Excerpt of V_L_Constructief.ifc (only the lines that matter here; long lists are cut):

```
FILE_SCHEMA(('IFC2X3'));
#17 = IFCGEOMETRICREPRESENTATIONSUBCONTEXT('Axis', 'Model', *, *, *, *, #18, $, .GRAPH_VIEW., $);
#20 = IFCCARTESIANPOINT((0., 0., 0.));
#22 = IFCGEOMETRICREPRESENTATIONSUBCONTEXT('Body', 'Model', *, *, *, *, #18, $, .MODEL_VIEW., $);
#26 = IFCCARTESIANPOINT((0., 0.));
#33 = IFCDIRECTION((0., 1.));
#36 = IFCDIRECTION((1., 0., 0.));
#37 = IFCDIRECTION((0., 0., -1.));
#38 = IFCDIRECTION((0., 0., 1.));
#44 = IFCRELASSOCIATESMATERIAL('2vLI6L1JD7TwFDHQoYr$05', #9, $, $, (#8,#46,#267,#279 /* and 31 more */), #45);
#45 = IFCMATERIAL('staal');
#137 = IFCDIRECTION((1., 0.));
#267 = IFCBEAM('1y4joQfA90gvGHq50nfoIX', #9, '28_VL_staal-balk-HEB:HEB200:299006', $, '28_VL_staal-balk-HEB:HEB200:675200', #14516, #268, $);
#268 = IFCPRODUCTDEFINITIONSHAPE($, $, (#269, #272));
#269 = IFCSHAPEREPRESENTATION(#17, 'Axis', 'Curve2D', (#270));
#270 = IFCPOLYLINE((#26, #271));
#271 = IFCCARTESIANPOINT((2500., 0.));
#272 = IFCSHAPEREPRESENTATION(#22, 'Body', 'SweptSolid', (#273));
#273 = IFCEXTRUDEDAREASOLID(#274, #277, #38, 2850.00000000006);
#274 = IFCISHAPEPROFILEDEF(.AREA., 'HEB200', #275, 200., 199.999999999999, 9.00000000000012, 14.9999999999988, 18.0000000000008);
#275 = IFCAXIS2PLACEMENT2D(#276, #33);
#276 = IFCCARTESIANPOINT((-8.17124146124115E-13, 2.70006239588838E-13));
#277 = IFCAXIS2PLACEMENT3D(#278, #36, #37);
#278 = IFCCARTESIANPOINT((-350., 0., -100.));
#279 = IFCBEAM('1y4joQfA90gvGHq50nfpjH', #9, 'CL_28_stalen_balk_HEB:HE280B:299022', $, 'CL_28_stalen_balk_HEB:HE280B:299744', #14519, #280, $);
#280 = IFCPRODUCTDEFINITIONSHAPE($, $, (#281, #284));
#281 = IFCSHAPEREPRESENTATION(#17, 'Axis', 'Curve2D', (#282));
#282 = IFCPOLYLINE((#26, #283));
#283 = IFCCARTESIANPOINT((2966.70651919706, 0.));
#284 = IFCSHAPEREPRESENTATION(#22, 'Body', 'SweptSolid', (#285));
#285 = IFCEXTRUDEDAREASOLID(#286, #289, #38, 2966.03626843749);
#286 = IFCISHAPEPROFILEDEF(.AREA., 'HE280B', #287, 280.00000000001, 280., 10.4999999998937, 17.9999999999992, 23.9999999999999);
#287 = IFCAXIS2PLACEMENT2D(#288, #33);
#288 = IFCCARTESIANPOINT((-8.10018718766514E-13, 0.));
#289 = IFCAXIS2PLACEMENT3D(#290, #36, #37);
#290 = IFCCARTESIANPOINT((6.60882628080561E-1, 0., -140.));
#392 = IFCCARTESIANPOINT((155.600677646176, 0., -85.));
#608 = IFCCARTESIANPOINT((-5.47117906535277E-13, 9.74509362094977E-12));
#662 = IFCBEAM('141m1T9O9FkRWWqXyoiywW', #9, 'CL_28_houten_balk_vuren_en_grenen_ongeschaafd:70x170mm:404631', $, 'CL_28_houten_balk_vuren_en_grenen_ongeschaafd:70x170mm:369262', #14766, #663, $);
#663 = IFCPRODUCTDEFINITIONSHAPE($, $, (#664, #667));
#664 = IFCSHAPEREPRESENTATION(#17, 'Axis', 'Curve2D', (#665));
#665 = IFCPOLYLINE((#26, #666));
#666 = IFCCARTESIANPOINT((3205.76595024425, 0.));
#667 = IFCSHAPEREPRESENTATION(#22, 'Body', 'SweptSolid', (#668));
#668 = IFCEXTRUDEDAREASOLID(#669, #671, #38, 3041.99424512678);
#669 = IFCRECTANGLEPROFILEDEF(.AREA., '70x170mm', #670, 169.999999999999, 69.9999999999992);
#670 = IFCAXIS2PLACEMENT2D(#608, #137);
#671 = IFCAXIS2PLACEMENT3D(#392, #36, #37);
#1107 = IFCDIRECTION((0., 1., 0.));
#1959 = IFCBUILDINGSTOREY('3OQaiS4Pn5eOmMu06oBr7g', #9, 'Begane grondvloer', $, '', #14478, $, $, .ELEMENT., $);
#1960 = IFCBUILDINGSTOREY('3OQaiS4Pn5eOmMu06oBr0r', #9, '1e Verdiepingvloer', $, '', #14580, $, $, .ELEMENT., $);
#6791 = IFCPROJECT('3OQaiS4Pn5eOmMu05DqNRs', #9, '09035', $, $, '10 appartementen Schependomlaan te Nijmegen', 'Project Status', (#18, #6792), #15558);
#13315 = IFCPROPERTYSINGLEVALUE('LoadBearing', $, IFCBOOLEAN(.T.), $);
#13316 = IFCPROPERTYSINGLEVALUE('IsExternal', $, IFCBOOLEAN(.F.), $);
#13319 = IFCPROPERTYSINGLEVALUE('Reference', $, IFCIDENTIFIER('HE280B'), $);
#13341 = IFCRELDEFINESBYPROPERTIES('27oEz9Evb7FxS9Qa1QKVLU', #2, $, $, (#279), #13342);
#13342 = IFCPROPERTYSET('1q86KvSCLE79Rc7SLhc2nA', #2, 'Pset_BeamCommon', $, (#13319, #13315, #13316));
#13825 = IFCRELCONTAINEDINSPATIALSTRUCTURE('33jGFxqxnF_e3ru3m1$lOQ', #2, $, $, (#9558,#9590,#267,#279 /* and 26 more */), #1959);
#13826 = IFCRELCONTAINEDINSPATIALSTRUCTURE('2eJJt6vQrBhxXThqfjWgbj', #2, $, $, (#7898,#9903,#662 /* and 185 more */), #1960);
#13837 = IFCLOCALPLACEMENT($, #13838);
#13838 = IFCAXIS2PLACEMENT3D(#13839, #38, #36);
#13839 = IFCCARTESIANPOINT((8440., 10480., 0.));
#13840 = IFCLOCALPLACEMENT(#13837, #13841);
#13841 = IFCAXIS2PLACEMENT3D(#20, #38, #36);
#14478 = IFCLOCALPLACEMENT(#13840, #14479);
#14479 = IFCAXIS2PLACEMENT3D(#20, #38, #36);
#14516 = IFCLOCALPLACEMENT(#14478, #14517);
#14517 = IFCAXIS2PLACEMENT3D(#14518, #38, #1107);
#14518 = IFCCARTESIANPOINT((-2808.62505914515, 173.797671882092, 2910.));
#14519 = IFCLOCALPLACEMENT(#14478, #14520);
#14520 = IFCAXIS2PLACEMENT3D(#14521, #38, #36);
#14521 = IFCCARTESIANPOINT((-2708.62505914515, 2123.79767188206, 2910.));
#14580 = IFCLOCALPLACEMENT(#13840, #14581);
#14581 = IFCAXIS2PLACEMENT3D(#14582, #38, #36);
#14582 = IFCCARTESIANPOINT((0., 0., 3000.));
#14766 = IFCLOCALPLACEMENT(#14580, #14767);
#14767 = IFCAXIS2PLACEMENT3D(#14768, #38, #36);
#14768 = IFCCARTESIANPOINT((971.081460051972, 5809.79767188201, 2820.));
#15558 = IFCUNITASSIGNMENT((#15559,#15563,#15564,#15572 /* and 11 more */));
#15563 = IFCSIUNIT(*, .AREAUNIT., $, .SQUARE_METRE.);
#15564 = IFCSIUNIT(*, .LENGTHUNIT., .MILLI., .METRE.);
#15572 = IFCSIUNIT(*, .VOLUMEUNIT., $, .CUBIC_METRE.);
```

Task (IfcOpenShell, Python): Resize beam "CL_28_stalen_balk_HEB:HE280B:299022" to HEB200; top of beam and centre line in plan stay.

```python
import ifcopenshell
import ifcopenshell.api.pset
import ifcopenshell.util.element
import ifcopenshell.util.representation

model = ifcopenshell.open("V_L_Constructief.ifc")

member = model.by_id(279)
source = next(p for p in model.by_type("IfcIShapeProfileDef") if p.ProfileName == "HEB200")

body = ifcopenshell.util.representation.get_representation(member, "Model", "Body")
solid = body.Items[0]
old_profile = solid.SweptArea

# Copy the section's sizes but keep this member's own profile position.
profile = ifcopenshell.util.element.copy(model, source)
# Profiles are centred, so shift by half the change in depth to hold the top.
shift = (old_profile.OverallDepth - profile.OverallDepth) / 2
x, y = old_profile.Position.Location.Coordinates
up = (-1.0, 0.0)  # upwards, in the solid's own plane
location = model.createIfcCartesianPoint((x + up[0] * shift, y + up[1] * shift))
profile.Position = model.createIfcAxis2Placement2D(location, old_profile.Position.RefDirection)
solid.SweptArea = profile
if not model.get_total_inverses(old_profile):
    ifcopenshell.util.element.remove_deep2(model, old_profile)
member.Name = member.Name.replace("HE280B", "HEB200")
member.ObjectType = member.ObjectType.replace("HE280B", "HEB200")
pset = model.by_id(ifcopenshell.util.element.get_pset(member, "Pset_BeamCommon", should_inherit=False)["id"])
ifcopenshell.api.pset.edit_pset(model, pset=pset, properties={"Reference": "HEB200"})

print(solid.SweptArea)

model.write("V_L_Constructief_updated.ifc")
```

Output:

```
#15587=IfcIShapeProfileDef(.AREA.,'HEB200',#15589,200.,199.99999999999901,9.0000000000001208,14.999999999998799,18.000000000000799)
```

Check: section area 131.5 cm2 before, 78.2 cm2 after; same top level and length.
